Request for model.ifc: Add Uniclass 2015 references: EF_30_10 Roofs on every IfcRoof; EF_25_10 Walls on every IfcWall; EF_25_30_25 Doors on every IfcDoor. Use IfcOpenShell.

First a look at what the model holds.

```python
import ifcopenshell

model = ifcopenshell.open("model.ifc")
print(model.schema)
print("classifications:", [c.Name for c in model.by_type("IfcClassification")])
for ifc_class in ("IfcDoor", "IfcRoof", "IfcStair", "IfcWall", "IfcWindow"):
    print(ifc_class, len(model.by_type(ifc_class)))
```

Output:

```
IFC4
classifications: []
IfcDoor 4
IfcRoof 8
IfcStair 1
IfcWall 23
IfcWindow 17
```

```python
import ifcopenshell
import ifcopenshell.api.classification

model = ifcopenshell.open("model.ifc")

system = ifcopenshell.api.classification.add_classification(model, classification="Uniclass 2015")

codes = {
    "IfcRoof": ("EF_30_10", "Roofs"),
    "IfcWall": ("EF_25_10", "Walls"),
    "IfcDoor": ("EF_25_30_25", "Doors"),
}
for ifc_class, (code, name) in codes.items():
    products = model.by_type(ifc_class)
    ifcopenshell.api.classification.add_reference(
        model, products=products, classification=system, identification=code, name=name
    )
    print(code, len(products))

model.write("model_v2.ifc")
```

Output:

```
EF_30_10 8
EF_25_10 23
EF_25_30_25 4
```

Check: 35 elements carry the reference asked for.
